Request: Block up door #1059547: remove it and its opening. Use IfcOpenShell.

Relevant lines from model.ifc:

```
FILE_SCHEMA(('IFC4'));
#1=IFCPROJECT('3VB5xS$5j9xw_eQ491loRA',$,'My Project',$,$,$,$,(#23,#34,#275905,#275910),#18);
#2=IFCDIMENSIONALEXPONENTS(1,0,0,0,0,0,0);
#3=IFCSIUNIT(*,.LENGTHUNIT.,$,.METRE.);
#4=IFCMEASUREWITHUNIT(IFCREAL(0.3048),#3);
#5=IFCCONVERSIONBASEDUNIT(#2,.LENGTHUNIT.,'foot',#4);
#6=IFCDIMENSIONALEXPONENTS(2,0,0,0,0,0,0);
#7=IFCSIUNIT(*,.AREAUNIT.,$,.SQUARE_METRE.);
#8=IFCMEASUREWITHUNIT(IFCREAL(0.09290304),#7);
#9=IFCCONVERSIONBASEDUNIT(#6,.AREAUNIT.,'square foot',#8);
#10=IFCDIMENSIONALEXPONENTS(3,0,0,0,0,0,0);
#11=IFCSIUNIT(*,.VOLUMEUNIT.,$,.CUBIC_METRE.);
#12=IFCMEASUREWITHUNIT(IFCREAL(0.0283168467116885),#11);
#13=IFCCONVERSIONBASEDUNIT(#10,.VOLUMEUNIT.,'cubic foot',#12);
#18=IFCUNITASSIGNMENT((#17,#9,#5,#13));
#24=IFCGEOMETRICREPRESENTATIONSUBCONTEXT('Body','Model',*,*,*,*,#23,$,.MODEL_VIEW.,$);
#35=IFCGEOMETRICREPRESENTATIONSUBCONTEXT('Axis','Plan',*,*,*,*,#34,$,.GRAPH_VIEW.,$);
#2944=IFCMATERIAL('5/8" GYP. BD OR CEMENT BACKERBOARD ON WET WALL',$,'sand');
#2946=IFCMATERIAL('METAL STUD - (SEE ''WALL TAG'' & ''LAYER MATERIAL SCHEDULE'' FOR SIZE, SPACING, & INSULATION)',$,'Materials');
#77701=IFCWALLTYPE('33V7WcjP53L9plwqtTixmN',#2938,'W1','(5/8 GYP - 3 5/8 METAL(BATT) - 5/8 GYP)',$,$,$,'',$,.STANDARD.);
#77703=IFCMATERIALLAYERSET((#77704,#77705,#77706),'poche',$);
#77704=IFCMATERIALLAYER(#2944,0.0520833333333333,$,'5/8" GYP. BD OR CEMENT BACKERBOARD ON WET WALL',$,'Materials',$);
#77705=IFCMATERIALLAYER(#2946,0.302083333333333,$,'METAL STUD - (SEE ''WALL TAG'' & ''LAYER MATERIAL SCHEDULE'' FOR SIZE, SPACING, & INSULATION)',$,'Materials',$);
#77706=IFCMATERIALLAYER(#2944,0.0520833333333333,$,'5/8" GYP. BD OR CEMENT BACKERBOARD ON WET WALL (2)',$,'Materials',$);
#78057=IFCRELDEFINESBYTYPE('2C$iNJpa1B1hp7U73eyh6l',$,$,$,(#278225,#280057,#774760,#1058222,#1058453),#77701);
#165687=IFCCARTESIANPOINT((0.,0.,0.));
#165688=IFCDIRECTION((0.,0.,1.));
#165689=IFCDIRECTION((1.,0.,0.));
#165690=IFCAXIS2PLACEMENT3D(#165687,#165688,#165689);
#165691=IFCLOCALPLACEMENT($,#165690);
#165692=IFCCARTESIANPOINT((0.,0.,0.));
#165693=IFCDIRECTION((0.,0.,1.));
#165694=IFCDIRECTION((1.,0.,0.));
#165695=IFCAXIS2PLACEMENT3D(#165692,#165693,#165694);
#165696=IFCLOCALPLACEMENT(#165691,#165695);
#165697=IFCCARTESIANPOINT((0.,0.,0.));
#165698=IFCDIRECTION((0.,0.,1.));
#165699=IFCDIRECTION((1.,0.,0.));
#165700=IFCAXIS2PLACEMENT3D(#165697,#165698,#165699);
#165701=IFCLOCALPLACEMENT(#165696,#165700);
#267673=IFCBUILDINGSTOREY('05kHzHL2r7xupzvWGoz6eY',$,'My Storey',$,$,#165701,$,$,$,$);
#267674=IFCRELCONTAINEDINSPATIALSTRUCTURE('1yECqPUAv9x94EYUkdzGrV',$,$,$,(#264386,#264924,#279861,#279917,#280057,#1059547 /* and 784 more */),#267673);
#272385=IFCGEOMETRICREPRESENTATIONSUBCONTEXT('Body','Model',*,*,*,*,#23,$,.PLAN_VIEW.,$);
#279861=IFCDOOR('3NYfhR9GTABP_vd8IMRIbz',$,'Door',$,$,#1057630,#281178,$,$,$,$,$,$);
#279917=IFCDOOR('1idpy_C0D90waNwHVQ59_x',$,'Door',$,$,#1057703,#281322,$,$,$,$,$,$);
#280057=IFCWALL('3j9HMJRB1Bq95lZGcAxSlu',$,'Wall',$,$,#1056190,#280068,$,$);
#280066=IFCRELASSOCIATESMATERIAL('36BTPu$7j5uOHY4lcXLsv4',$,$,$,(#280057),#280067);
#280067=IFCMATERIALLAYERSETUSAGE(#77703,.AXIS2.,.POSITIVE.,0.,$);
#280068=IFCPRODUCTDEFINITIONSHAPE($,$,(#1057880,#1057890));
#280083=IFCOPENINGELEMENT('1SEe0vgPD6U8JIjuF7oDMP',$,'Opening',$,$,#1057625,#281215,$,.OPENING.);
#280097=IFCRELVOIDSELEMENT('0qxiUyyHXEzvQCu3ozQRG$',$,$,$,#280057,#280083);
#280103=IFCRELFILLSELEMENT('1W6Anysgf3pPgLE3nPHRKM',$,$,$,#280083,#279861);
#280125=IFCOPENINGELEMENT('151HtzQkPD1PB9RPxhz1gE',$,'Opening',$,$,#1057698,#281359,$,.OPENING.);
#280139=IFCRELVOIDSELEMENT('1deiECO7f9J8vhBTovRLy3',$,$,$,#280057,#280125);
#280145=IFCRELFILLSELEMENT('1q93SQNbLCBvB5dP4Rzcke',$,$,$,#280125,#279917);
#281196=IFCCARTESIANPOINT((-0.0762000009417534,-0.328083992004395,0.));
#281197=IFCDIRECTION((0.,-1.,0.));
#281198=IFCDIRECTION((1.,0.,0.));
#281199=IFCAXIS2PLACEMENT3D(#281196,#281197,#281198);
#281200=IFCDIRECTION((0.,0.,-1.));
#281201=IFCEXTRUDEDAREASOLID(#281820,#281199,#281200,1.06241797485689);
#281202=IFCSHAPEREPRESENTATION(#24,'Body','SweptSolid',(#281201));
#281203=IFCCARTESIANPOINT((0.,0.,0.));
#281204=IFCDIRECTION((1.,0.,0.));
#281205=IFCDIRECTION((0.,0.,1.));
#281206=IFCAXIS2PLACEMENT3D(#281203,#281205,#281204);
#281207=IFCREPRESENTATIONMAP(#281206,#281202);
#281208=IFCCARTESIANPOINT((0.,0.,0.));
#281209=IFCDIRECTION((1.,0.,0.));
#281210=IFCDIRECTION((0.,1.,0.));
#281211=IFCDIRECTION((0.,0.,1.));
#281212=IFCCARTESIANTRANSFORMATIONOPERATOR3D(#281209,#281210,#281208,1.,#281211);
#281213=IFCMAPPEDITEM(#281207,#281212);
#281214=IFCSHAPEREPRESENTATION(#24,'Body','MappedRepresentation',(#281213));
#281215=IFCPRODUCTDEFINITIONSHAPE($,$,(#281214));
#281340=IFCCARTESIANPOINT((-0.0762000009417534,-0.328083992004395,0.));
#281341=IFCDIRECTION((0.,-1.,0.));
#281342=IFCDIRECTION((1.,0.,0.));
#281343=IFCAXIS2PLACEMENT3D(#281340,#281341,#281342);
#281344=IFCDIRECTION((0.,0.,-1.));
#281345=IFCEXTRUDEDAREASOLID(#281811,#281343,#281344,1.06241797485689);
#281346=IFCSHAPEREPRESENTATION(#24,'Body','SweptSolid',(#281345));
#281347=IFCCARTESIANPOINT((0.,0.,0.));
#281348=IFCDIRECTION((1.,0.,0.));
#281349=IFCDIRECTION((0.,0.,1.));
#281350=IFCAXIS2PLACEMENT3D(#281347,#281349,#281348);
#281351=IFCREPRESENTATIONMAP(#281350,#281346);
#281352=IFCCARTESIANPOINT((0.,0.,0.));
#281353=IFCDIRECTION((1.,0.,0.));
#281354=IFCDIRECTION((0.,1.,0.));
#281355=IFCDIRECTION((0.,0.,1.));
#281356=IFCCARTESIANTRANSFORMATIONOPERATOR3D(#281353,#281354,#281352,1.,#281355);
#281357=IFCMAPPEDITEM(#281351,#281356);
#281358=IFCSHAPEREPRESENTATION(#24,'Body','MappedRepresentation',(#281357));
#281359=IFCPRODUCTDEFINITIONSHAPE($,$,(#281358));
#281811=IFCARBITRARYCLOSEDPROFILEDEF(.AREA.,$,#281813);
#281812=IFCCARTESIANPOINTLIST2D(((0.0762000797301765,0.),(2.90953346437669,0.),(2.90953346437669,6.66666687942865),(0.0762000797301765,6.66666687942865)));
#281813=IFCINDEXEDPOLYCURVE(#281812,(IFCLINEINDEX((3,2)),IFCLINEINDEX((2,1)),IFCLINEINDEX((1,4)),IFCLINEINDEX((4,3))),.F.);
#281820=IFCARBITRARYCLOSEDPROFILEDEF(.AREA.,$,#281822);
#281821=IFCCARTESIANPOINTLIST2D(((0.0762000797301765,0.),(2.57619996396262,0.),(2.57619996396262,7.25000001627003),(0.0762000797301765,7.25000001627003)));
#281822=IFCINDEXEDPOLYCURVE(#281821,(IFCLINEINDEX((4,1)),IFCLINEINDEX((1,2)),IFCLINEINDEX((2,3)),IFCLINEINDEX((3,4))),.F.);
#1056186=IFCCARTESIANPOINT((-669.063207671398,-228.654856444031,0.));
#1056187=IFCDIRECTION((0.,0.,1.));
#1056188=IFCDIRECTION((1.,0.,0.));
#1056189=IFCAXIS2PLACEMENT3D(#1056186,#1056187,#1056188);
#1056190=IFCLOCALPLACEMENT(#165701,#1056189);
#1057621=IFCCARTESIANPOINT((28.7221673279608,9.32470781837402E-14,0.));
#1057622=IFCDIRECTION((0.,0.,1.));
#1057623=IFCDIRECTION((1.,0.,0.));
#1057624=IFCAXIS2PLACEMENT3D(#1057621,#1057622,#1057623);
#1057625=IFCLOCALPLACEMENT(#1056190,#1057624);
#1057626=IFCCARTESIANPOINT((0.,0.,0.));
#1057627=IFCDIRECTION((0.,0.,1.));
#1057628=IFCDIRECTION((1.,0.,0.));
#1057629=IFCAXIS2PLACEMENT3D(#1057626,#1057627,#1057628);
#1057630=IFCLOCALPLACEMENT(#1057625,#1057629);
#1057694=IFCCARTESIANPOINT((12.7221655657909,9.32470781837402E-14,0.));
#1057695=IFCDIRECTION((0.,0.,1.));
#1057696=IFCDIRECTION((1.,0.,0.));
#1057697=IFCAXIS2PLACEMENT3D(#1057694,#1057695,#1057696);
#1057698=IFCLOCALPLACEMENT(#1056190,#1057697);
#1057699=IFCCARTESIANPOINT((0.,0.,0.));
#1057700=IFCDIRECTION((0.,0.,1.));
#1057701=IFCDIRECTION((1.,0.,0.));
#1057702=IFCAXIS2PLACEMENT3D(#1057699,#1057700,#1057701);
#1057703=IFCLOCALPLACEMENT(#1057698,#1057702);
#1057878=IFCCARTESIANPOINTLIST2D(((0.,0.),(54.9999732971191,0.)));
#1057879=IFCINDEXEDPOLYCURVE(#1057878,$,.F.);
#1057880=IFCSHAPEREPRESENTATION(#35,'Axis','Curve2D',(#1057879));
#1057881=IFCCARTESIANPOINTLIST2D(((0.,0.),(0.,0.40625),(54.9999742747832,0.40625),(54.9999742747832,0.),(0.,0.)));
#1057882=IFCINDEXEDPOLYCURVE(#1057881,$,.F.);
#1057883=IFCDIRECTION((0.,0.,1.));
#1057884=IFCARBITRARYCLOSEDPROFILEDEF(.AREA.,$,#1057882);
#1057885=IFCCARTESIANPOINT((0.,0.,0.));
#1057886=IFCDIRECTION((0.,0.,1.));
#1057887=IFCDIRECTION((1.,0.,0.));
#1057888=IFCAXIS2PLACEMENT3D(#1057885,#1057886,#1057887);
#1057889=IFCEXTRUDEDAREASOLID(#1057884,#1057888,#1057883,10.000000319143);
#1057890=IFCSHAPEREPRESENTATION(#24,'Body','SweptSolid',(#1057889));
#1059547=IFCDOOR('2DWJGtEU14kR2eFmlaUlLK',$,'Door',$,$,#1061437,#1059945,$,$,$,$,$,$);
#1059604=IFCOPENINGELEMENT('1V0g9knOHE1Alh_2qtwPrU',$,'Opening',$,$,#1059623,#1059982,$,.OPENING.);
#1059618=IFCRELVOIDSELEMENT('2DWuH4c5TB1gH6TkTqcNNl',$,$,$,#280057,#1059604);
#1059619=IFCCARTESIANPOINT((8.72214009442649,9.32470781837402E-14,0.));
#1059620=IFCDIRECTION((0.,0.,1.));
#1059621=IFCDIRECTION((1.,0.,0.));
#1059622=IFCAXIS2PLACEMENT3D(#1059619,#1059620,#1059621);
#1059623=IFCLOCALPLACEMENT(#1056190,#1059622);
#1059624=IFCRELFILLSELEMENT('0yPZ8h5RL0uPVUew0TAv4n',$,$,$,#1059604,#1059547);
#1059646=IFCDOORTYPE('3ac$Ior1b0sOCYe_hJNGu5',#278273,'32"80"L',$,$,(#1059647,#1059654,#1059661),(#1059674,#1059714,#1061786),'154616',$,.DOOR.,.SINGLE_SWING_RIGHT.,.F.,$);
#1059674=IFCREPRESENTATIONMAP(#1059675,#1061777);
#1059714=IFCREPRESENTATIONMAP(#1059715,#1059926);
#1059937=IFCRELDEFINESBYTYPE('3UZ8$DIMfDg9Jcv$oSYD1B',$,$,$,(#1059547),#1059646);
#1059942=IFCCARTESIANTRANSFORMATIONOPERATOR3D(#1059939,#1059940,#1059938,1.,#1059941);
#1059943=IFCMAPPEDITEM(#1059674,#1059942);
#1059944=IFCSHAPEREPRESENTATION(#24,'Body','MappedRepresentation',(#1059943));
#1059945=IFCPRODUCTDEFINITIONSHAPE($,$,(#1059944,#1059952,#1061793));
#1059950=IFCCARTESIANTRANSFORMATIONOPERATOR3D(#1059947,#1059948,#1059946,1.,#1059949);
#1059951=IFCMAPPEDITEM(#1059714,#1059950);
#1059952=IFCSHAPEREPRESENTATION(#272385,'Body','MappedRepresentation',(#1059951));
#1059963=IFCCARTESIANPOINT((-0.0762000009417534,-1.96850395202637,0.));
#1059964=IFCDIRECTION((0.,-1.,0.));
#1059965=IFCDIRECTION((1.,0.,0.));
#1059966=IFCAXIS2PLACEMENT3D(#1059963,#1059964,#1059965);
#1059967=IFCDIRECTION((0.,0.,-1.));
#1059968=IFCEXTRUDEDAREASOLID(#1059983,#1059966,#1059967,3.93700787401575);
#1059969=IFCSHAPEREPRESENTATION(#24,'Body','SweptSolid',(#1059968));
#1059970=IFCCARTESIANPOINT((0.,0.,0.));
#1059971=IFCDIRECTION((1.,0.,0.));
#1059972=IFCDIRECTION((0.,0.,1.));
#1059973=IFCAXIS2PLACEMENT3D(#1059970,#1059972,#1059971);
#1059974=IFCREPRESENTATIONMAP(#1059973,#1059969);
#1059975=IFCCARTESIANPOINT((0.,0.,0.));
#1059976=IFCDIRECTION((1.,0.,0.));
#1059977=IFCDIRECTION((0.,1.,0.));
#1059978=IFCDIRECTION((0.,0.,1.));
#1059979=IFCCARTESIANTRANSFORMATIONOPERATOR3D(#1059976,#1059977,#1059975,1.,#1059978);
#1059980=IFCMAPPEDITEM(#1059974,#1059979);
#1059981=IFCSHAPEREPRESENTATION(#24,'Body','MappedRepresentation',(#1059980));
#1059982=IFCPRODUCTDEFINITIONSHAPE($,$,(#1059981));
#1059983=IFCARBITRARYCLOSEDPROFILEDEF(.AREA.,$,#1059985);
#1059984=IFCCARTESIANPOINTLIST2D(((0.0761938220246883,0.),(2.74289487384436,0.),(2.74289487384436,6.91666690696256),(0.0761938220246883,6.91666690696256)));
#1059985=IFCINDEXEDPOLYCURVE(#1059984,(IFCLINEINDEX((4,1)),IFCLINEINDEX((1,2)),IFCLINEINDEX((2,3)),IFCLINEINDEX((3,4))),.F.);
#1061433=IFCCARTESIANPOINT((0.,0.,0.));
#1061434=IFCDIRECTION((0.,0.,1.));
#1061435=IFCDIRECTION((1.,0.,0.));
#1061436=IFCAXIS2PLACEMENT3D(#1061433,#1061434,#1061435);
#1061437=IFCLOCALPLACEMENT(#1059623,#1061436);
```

```python
import ifcopenshell
import ifcopenshell.api.feature
import ifcopenshell.api.root
import ifcopenshell.geom
import ifcopenshell.util.shape

model = ifcopenshell.open("model.ifc")
settings = ifcopenshell.geom.settings()


def volume(element):
    """Net volume in cubic metres, openings subtracted."""
    shape = ifcopenshell.geom.create_shape(settings, element)
    return ifcopenshell.util.shape.get_volume(shape.geometry)


door = model.by_guid("2DWJGtEU14kR2eFmlaUlLK")
opening = door.FillsVoids[0].RelatingOpeningElement
wall = opening.VoidsElements[0].RelatingBuildingElement
before = volume(wall)

ifcopenshell.api.root.remove_product(model, product=door)
ifcopenshell.api.feature.remove_feature(model, feature=opening)

after = volume(wall)

print(f"wall volume {before:.3f} -> {after:.3f} m3")

model.write("model_rev.ifc")
```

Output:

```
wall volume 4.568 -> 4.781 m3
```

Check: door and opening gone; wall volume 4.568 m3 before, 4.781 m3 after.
